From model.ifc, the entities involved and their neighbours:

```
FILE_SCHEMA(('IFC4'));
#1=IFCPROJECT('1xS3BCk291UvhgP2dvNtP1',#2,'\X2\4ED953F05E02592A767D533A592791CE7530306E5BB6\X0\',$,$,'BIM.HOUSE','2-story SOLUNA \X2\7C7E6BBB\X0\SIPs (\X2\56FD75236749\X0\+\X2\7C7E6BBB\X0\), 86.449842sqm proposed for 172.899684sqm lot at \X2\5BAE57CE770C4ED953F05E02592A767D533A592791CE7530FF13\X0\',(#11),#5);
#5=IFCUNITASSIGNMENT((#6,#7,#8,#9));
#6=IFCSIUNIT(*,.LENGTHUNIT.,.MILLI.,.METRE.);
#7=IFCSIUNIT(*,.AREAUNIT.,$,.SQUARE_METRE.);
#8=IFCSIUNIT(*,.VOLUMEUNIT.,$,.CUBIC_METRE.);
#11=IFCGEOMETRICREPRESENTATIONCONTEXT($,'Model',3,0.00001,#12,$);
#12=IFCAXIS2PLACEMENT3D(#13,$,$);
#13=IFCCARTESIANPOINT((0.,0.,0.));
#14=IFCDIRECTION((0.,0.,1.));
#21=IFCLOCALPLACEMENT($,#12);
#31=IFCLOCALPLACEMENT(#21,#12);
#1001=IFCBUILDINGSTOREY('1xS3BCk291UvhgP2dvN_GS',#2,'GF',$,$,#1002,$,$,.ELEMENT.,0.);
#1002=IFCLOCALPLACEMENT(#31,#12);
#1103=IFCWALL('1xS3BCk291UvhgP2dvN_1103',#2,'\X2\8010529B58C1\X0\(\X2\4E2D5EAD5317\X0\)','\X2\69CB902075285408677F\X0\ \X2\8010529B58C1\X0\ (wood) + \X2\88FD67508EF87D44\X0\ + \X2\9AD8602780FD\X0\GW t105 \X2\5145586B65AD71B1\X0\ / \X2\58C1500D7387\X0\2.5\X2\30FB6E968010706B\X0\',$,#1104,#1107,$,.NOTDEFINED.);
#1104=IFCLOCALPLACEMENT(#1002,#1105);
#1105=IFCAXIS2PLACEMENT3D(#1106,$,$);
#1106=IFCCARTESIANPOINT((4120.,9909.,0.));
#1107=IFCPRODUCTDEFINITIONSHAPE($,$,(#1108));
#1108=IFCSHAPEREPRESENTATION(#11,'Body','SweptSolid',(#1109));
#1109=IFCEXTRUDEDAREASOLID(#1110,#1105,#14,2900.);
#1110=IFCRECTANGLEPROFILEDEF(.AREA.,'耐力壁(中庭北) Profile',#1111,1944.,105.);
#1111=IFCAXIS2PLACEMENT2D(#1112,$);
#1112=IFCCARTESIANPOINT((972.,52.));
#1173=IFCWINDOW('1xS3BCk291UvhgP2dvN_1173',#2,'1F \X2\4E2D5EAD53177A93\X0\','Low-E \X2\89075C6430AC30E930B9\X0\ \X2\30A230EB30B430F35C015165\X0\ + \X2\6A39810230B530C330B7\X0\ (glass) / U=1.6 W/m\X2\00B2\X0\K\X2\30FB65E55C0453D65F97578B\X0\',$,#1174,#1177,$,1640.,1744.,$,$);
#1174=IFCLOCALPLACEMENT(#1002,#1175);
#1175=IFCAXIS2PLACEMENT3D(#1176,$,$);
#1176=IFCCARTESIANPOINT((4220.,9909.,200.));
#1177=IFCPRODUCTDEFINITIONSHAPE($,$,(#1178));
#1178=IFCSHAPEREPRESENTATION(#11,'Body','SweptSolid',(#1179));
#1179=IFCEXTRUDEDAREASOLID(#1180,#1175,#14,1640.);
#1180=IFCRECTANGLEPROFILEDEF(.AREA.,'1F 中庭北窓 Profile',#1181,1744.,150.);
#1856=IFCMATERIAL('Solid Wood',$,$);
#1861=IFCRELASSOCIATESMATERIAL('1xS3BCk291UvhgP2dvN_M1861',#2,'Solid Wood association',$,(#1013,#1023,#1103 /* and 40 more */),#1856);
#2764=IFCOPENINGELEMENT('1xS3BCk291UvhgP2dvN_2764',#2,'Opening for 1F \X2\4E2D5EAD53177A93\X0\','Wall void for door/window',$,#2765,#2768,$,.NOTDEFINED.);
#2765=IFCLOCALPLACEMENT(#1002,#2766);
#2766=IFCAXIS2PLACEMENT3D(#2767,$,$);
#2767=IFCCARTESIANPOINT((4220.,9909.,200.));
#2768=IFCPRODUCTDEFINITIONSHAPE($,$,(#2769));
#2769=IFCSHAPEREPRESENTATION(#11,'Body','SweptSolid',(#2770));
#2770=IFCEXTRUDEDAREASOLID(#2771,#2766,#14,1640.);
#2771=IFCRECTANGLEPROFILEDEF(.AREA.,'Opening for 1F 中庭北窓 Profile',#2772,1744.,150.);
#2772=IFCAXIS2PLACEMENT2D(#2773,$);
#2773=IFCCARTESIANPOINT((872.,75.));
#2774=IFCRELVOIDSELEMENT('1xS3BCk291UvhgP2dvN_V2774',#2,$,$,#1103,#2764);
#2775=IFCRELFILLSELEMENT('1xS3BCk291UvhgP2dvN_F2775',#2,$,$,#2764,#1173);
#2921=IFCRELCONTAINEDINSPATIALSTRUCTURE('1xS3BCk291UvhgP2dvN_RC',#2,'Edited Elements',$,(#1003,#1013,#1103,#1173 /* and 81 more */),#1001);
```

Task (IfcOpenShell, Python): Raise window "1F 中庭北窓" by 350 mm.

```python
import numpy as np
import ifcopenshell
import ifcopenshell.api.geometry
import ifcopenshell.util.placement
import ifcopenshell.util.unit

model = ifcopenshell.open("model.ifc")
unit_scale = ifcopenshell.util.unit.calculate_unit_scale(model)

window = model.by_id(1173)
opening = window.FillsVoids[0].RelatingOpeningElement
dz = 350.0

shift = np.array([0.0, 0.0, dz])
# The window is not placed relative to its opening, so move both.
for product in (opening, window):
    matrix = ifcopenshell.util.placement.get_local_placement(product.ObjectPlacement)
    matrix[:3, 3] += shift
    ifcopenshell.api.geometry.edit_object_placement(model, product=product, matrix=matrix, is_si=False)

print(f"moved by {dz * unit_scale:+.3f} m")

model.write("model-out.ifc")
```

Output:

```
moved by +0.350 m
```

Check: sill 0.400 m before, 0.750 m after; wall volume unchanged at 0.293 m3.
